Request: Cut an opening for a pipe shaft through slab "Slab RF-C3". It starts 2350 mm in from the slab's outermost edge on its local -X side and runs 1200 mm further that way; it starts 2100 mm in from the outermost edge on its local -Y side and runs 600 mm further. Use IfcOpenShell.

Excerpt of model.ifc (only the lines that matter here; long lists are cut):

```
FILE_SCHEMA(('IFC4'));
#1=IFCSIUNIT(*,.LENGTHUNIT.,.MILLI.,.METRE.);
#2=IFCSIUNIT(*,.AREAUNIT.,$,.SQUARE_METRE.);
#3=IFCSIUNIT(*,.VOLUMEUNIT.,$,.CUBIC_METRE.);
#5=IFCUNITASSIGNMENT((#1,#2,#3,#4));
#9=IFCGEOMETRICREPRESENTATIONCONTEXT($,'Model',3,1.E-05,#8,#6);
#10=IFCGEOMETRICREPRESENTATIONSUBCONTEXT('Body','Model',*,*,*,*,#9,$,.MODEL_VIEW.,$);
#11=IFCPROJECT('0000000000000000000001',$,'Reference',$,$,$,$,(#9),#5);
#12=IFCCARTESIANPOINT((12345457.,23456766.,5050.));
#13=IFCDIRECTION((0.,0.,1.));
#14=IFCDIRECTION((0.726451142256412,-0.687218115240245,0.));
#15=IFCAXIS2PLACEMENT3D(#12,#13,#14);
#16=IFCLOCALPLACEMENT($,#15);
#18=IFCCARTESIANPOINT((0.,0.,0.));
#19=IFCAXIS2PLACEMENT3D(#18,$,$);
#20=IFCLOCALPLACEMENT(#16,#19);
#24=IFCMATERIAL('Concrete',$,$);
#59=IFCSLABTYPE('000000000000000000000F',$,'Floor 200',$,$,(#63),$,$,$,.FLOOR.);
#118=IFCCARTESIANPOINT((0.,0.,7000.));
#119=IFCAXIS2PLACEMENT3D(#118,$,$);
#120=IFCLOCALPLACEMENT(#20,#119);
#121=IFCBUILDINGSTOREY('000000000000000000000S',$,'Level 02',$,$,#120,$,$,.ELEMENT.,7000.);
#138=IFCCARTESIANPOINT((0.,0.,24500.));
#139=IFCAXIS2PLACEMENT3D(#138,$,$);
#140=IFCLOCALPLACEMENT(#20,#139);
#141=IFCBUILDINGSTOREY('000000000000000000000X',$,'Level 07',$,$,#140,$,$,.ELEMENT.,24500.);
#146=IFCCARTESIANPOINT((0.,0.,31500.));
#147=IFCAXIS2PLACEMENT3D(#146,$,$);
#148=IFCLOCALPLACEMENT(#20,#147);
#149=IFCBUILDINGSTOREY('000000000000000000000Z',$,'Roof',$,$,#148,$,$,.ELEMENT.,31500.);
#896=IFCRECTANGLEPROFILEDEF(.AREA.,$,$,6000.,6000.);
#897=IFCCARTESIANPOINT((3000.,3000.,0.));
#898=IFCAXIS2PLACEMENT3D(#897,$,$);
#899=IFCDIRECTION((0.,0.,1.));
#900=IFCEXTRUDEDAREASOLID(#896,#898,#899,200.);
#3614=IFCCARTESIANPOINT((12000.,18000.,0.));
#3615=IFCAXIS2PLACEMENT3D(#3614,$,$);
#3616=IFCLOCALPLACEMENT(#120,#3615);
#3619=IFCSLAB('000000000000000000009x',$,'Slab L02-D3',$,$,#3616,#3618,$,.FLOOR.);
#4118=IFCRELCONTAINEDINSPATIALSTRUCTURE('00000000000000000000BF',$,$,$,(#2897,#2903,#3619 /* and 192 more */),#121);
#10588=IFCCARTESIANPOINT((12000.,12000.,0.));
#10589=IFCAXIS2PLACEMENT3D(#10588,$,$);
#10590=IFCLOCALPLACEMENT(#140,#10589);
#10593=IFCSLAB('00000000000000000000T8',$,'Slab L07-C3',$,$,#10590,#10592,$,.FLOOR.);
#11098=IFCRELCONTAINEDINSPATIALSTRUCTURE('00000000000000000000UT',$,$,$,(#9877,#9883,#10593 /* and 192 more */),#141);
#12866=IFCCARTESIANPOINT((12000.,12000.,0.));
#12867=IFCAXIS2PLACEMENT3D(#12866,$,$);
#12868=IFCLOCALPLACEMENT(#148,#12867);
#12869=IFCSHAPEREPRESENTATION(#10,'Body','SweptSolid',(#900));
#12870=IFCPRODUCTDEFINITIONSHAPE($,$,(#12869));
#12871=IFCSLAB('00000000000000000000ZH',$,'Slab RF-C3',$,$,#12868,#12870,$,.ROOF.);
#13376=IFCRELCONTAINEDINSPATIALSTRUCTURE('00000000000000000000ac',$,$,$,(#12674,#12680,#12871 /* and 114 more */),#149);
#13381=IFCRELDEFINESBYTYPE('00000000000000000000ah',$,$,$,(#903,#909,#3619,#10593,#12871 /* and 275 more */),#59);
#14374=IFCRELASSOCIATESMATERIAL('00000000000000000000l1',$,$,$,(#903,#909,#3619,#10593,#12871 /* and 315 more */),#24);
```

```python
import numpy as np
import ifcopenshell
import ifcopenshell.api.feature
import ifcopenshell.api.geometry
import ifcopenshell.api.root
import ifcopenshell.geom
import ifcopenshell.util.placement
import ifcopenshell.util.representation
import ifcopenshell.util.shape
import ifcopenshell.util.unit

model = ifcopenshell.open("model.ifc")
unit_scale = ifcopenshell.util.unit.calculate_unit_scale(model)
settings = ifcopenshell.geom.settings()


def volume(element):
    """Net volume in cubic metres, openings subtracted."""
    shape = ifcopenshell.geom.create_shape(settings, element)
    return ifcopenshell.util.shape.get_volume(shape.geometry)


slab = model.by_id(12871)
before = volume(slab)

# Extent in the slab's own axes, in metres. The edges named are its -X and -Y sides.
slab_shape = ifcopenshell.geom.create_shape(settings, slab)
vertices = ifcopenshell.util.shape.get_vertices(slab_shape.geometry)
x_min, y_min, bottom = vertices.min(axis=0)
top = vertices[:, 2].max()

opening = ifcopenshell.api.root.create_entity(model, ifc_class="IfcOpeningElement", name="Pipe shaft opening", predefined_type="OPENING")
context = ifcopenshell.util.representation.get_context(model, "Model", "Body", "MODEL_VIEW")
width, depth = 1.2, 0.6
outline = [(0.0, 0.0), (width, 0.0), (width, depth), (0.0, depth), (0.0, 0.0)]
# Overshoot both faces by 50 mm so the cut is clean.
shape = ifcopenshell.api.geometry.add_slab_representation(
    model, context=context, depth=top - bottom + 0.1, polyline=outline
)
ifcopenshell.api.geometry.assign_representation(model, product=opening, representation=shape)

matrix = ifcopenshell.util.placement.get_local_placement(slab.ObjectPlacement)
matrix[:, 3] = matrix @ np.append(np.array([x_min + 2.35, y_min + 2.1, bottom - 0.05]) / unit_scale, 1.0)
ifcopenshell.api.geometry.edit_object_placement(model, product=opening, matrix=matrix, is_si=False)
ifcopenshell.api.feature.add_feature(model, feature=opening, element=slab)

after = volume(slab)

print(f"slab volume {before:.3f} -> {after:.3f} m3")

model.write("model_updated.ifc")
```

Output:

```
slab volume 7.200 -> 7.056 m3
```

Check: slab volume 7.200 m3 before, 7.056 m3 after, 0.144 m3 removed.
